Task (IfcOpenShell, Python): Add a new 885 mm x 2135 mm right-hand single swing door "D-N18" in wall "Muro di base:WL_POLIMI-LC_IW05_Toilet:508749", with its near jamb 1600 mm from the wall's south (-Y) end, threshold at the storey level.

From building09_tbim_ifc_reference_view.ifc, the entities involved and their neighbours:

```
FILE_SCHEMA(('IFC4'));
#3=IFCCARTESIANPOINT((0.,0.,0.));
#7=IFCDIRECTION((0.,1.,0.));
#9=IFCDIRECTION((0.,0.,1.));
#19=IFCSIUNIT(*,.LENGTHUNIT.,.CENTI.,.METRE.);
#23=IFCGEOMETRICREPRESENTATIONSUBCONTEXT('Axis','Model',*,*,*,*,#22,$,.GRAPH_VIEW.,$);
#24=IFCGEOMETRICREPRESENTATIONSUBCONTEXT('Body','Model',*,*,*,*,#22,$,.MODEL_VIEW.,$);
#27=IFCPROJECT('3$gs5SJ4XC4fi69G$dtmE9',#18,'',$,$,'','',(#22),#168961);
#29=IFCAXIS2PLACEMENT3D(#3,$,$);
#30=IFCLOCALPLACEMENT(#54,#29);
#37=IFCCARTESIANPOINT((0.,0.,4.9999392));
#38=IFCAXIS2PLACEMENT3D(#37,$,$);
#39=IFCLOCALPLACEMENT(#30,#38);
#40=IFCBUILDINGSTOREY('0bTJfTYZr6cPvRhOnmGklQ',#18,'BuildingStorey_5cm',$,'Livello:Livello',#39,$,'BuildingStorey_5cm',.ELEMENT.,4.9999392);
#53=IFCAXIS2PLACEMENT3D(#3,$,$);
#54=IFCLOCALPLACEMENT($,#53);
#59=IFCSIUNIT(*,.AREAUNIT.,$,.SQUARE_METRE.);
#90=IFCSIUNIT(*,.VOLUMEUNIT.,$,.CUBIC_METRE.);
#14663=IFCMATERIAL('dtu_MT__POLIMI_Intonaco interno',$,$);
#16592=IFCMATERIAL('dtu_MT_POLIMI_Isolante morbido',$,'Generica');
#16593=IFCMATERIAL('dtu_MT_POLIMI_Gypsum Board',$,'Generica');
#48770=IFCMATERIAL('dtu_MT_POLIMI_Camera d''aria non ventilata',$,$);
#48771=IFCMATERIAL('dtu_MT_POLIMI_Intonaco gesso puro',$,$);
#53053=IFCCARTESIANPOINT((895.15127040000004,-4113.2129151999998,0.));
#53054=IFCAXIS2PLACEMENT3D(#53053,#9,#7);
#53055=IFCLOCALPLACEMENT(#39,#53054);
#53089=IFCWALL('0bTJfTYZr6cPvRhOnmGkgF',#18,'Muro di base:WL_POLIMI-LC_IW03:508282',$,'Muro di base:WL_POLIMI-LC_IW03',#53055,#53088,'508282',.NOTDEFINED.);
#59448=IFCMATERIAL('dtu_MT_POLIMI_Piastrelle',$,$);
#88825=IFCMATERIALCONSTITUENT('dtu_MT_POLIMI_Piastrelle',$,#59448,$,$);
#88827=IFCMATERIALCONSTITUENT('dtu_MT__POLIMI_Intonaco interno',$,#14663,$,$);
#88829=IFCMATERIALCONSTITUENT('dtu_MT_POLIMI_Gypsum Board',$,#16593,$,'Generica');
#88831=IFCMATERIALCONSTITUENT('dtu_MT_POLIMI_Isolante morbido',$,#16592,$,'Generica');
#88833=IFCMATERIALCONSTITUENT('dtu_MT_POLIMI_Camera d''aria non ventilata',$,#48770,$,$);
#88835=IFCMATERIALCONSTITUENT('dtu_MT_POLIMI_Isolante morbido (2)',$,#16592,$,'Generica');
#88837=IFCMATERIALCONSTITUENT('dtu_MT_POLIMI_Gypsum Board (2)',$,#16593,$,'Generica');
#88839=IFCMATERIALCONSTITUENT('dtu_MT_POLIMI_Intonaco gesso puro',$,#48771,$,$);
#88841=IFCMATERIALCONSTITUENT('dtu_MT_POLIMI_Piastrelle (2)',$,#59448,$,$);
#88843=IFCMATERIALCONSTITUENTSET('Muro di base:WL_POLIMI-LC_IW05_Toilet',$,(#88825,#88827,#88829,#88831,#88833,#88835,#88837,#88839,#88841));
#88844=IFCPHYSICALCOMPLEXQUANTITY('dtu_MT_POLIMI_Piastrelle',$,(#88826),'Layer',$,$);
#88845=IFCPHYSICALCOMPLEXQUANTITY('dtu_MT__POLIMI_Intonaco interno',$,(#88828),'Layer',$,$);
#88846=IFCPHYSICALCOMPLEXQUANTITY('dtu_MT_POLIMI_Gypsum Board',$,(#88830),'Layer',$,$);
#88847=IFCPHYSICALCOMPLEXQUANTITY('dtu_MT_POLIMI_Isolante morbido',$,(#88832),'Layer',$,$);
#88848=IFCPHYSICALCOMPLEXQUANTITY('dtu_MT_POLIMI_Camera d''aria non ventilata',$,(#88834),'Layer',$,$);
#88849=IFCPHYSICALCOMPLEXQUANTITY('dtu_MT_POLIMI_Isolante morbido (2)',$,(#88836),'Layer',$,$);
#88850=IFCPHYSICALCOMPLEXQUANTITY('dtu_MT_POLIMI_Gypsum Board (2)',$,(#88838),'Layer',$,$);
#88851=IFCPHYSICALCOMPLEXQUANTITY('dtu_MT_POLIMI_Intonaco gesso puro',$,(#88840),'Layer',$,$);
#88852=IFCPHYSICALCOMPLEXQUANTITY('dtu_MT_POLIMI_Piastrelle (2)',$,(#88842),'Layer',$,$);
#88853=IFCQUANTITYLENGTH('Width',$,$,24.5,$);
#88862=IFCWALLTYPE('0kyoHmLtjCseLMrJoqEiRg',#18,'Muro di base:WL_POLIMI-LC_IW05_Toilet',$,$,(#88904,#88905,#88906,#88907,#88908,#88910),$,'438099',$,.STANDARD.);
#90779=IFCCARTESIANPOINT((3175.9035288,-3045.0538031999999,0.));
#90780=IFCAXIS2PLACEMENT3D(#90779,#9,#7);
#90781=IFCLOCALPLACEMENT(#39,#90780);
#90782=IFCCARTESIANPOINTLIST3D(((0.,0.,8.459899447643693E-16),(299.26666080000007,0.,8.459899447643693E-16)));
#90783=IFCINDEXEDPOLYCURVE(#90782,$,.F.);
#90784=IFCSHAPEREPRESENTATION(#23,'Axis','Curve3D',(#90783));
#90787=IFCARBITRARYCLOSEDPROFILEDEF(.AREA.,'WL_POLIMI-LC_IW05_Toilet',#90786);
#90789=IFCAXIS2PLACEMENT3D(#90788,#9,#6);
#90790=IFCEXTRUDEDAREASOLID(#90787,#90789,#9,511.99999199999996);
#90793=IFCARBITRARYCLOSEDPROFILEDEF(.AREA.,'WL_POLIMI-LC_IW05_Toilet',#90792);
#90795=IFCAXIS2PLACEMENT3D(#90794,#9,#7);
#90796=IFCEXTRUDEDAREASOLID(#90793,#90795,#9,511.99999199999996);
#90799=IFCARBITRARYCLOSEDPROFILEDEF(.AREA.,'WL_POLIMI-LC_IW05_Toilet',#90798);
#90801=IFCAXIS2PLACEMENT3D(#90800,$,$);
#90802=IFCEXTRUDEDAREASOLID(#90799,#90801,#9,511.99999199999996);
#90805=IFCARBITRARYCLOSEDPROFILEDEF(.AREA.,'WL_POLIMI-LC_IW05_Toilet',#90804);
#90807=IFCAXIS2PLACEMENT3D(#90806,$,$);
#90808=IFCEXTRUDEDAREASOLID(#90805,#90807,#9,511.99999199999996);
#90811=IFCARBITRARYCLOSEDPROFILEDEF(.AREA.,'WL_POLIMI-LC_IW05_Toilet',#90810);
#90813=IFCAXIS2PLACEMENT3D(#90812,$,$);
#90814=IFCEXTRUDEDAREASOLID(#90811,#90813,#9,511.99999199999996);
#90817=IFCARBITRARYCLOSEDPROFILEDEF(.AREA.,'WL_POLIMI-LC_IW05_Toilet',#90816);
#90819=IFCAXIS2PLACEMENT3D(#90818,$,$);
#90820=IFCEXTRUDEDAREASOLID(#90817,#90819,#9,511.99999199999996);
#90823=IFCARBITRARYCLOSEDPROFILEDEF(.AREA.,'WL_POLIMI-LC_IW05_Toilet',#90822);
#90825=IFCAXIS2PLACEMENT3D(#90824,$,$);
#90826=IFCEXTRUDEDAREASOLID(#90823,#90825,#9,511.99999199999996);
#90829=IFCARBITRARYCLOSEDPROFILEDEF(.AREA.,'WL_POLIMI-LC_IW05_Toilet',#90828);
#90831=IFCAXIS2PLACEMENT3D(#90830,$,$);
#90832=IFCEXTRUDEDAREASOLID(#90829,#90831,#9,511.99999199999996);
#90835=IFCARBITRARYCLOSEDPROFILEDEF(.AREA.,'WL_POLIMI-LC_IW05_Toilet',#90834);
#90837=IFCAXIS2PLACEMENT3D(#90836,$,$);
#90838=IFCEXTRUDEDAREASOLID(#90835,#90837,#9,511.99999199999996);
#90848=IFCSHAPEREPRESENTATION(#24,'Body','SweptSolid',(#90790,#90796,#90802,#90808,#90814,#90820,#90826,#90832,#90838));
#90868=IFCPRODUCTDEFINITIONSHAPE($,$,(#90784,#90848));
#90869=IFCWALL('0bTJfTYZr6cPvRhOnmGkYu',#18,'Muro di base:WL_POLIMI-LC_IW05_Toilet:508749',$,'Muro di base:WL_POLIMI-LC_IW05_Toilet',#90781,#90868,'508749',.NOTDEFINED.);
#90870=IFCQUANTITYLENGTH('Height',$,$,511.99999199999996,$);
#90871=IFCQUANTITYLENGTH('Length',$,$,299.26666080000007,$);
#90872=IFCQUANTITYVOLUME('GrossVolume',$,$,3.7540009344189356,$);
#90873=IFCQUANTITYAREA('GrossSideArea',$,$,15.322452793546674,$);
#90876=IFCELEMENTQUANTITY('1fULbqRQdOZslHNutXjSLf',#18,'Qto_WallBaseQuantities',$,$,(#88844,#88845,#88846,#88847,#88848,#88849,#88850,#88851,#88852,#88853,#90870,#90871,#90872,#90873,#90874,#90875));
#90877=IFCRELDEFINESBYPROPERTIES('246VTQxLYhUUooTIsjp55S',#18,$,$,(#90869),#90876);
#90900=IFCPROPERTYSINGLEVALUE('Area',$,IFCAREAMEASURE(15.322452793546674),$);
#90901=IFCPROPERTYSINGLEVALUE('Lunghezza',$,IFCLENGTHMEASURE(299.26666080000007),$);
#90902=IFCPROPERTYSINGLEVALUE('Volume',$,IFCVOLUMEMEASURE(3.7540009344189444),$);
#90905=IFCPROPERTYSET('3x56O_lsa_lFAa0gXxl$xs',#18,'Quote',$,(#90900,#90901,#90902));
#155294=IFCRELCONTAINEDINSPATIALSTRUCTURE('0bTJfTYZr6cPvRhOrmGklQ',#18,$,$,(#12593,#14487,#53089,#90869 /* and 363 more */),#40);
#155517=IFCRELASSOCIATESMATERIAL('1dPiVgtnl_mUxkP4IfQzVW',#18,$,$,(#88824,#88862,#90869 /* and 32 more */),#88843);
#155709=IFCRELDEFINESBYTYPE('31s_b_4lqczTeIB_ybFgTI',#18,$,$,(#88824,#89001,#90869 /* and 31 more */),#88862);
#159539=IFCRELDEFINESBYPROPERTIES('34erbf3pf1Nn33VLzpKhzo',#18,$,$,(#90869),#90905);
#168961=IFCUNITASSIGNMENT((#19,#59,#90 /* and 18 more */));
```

```python
import numpy as np
import ifcopenshell
import ifcopenshell.api.feature
import ifcopenshell.api.geometry
import ifcopenshell.api.pset
import ifcopenshell.api.root
import ifcopenshell.api.spatial
import ifcopenshell.geom
import ifcopenshell.util.element
import ifcopenshell.util.placement
import ifcopenshell.util.representation
import ifcopenshell.util.shape
import ifcopenshell.util.unit

model = ifcopenshell.open("building09_tbim_ifc_reference_view.ifc")
unit_scale = ifcopenshell.util.unit.calculate_unit_scale(model)
area_scale = ifcopenshell.util.unit.calculate_unit_scale(model, "AREAUNIT")
volume_scale = ifcopenshell.util.unit.calculate_unit_scale(model, "VOLUMEUNIT")
settings = ifcopenshell.geom.settings()


def volume(element):
    """Net volume in cubic metres, openings subtracted."""
    shape = ifcopenshell.geom.create_shape(settings, element)
    return ifcopenshell.util.shape.get_volume(shape.geometry)


wall = model.by_guid("0bTJfTYZr6cPvRhOnmGkYu")
storey = ifcopenshell.util.element.get_container(wall, ifc_class="IfcBuildingStorey")
context = ifcopenshell.util.representation.get_context(model, "Model", "Body", "MODEL_VIEW")
before = volume(wall)

width, height, from_end, sill = 0.885, 2.135, 1.6, 0.0  # metres

# The wall runs along its own X axis, and the end named is its -X end.
wall_shape = ifcopenshell.geom.create_shape(settings, wall)
x, y, z = ifcopenshell.util.shape.get_vertices(wall_shape.geometry).T
start = x.min() + from_end
face, thickness = float(y.min()), float(y.max() - y.min())
wall_matrix = ifcopenshell.util.placement.get_local_placement(wall.ObjectPlacement)
level = ifcopenshell.util.placement.get_local_placement(storey.ObjectPlacement)[2, 3]


def in_wall(x, y):
    """Placement at x, y metres in the wall's axes, at sill height."""
    matrix = wall_matrix.copy()
    matrix[:, 3] = wall_matrix @ np.array([x / unit_scale, y / unit_scale, 0.0, 1.0])
    matrix[2, 3] = level + sill / unit_scale
    return matrix


# Opening: a box that overshoots both wall faces by 50 mm.
opening = ifcopenshell.api.root.create_entity(model, ifc_class="IfcOpeningElement", predefined_type="OPENING")
box = ifcopenshell.api.geometry.add_wall_representation(
    model, context=context, length=width, height=height, thickness=thickness + 0.1
)
ifcopenshell.api.geometry.assign_representation(model, product=opening, representation=box)
ifcopenshell.api.geometry.edit_object_placement(model, product=opening, matrix=in_wall(start, face - 0.05), is_si=False)
ifcopenshell.api.feature.add_feature(model, feature=opening, element=wall)

door = ifcopenshell.api.root.create_entity(model, ifc_class="IfcDoor", name="D-N18", predefined_type="DOOR")
door.OverallWidth, door.OverallHeight = width / unit_scale, height / unit_scale
door.OperationType = "SINGLE_SWING_RIGHT"
body = ifcopenshell.api.geometry.add_door_representation(
    model,
    context=context,
    overall_width=door.OverallWidth,
    overall_height=door.OverallHeight,
    operation_type="SINGLE_SWING_RIGHT",
    lining_properties={"LiningDepth": thickness / unit_scale, "ThresholdDepth": thickness / unit_scale},
)
ifcopenshell.api.geometry.assign_representation(model, product=door, representation=body)
ifcopenshell.api.spatial.assign_container(model, products=[door], relating_structure=storey)
ifcopenshell.api.feature.add_filling(model, opening=opening, element=door)

# The lining spans the wall, so the door starts at the wall face.
ifcopenshell.api.geometry.edit_object_placement(model, product=door, matrix=in_wall(start, face), is_si=False)

after = volume(wall)

# Update the wall's stored quantities.
qto = model.by_id(ifcopenshell.util.element.get_pset(wall, "Qto_WallBaseQuantities", should_inherit=False)["id"])
ifcopenshell.api.pset.edit_qto(model, qto=qto, properties={
    "NetSideArea": after / thickness / area_scale,
    "NetVolume": after / volume_scale,
})
pset = model.by_id(ifcopenshell.util.element.get_pset(wall, "Quote", should_inherit=False)["id"])
ifcopenshell.api.pset.edit_pset(model, pset=pset, properties={
    "Area": model.create_entity("IfcAreaMeasure", after / thickness / area_scale),
    "Volume": model.create_entity("IfcVolumeMeasure", after / volume_scale),
})

print(f"wall volume {before:.3f} -> {after:.3f} m3")

model.write("building09_tbim_ifc_reference_view_edited.ifc")
```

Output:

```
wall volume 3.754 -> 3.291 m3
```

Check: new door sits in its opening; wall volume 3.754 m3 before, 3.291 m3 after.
